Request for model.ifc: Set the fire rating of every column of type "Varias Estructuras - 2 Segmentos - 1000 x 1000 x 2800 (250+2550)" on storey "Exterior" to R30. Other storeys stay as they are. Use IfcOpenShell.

First a look at what the model holds.

```python
import ifcopenshell
import ifcopenshell.util.element

model = ifcopenshell.open("model.ifc")
print(model.schema)
storey = next(s for s in model.by_type("IfcBuildingStorey") if s.Name == "Exterior")
columns = [e for e in ifcopenshell.util.element.get_decomposition(storey) if e.is_a("IfcColumn")]
seen = {}
for e in columns:
    element_type = ifcopenshell.util.element.get_type(e)
    key = (element_type.Name if element_type != e and element_type else None, ifcopenshell.util.element.get_pset(e, "Pset_ColumnCommon", "FireRating"))
    seen[key] = seen.get(key, 0) + 1
for (name, value), count in sorted(seen.items(), key=str):
    print(count, "x", name, "|", value)
```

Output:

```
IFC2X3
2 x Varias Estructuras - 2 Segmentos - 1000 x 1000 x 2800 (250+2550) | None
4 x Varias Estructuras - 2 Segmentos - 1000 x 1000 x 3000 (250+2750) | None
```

```python
import ifcopenshell
import ifcopenshell.api.pset
import ifcopenshell.util.element

model = ifcopenshell.open("model.ifc")

storey = next(s for s in model.by_type("IfcBuildingStorey") if s.Name == "Exterior")
columns = [e for e in ifcopenshell.util.element.get_decomposition(storey) if e.is_a("IfcColumn")]

count = 0
for e in columns:
    element_type = ifcopenshell.util.element.get_type(e)
    if element_type in (None, e) or element_type.Name != "Varias Estructuras - 2 Segmentos - 1000 x 1000 x 2800 (250+2550)":
        continue
    # add_pset returns the element's existing set when there is one.
    pset = ifcopenshell.api.pset.add_pset(model, product=e, name="Pset_ColumnCommon")
    ifcopenshell.api.pset.edit_pset(model, pset=pset, properties={"FireRating": "R30"})
    count += 1

print(count, "columns updated")

model.write("model_updated.ifc")
```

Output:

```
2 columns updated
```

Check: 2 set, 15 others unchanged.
